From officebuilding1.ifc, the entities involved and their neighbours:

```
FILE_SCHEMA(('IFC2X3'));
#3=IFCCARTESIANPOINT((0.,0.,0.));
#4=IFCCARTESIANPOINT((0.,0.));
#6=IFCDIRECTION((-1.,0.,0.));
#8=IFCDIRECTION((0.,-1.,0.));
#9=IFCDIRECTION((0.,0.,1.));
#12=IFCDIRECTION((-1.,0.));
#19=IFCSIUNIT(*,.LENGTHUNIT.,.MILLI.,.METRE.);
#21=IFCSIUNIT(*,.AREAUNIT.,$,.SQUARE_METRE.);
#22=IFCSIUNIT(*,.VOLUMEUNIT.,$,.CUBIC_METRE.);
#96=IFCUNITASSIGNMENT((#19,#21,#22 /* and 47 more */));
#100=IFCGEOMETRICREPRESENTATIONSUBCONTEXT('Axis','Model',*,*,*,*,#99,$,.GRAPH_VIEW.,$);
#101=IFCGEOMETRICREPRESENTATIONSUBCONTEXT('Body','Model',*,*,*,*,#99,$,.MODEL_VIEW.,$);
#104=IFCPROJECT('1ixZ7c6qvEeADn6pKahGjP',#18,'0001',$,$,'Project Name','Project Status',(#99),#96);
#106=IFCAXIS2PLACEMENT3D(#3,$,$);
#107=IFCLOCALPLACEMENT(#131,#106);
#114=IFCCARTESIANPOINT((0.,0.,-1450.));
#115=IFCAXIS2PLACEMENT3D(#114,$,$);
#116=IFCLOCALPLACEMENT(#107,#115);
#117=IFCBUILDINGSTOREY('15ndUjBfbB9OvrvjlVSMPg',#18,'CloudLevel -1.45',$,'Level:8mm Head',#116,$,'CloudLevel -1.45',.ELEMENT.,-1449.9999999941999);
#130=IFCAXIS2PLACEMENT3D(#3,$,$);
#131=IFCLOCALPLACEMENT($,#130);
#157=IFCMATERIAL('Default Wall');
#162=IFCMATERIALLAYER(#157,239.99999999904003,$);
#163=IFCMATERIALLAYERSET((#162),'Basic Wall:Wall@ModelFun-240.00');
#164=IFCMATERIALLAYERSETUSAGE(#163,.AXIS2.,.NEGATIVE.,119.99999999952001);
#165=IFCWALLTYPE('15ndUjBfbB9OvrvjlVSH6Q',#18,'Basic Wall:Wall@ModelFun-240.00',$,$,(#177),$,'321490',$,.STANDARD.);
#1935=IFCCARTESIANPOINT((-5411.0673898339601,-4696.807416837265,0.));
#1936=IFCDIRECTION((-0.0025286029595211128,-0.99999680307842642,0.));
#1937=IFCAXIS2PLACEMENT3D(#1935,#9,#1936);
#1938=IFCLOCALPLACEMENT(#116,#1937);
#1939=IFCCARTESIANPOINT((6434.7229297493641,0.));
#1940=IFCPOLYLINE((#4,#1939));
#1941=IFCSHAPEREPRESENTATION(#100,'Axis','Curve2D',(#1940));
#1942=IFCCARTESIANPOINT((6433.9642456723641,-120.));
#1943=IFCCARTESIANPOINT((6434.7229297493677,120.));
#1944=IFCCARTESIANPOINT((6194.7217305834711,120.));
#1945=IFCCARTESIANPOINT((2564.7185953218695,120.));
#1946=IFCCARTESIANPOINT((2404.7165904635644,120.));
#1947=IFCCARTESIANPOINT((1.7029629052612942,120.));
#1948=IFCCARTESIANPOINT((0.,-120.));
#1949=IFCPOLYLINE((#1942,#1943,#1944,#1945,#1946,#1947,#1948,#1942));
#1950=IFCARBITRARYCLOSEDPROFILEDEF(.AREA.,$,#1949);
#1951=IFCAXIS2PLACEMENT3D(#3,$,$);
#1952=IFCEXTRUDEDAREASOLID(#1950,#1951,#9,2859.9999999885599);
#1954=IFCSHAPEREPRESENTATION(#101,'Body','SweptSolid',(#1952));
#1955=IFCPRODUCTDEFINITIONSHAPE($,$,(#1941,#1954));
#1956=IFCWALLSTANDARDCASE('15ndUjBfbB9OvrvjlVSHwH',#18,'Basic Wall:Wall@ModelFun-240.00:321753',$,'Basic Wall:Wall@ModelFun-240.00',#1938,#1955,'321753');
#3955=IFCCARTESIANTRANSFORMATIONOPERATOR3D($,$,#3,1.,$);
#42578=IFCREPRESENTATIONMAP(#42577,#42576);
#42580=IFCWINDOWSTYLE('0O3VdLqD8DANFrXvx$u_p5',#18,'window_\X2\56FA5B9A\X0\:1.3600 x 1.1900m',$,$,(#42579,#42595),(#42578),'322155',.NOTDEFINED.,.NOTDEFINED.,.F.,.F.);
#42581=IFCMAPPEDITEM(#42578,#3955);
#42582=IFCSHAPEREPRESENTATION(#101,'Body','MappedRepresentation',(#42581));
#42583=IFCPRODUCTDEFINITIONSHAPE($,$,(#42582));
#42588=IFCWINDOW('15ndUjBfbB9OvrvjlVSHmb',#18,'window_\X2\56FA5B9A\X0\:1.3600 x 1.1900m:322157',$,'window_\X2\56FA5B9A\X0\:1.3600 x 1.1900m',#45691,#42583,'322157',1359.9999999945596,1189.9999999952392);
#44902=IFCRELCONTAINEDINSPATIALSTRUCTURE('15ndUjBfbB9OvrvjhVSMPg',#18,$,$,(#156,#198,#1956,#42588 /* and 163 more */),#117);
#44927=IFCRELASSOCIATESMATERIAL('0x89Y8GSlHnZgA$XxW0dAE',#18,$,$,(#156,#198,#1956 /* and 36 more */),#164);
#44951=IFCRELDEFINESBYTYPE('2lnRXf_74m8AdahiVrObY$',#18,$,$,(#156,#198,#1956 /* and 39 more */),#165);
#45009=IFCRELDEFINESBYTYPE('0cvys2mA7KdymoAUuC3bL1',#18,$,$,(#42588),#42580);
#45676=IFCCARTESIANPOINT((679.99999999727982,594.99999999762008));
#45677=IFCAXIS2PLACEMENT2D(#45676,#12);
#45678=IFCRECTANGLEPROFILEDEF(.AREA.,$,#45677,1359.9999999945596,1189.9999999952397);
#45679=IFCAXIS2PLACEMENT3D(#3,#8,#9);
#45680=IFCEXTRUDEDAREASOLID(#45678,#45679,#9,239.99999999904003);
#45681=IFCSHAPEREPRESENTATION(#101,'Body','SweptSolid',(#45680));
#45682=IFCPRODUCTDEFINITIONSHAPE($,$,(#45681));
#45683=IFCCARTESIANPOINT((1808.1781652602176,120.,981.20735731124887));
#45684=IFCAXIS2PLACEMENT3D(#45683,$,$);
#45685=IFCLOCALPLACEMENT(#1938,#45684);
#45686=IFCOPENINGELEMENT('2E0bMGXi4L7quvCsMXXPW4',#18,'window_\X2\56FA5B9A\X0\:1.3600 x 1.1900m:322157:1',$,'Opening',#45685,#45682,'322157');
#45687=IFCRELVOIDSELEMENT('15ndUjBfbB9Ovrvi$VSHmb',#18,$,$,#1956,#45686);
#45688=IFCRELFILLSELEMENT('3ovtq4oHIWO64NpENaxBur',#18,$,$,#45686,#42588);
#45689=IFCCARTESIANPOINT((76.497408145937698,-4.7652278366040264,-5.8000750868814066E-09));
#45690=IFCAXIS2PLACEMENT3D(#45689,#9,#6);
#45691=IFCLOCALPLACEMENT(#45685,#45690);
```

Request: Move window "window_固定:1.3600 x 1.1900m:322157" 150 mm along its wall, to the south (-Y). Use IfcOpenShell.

```python
import ifcopenshell
import ifcopenshell.api.geometry
import ifcopenshell.util.placement

model = ifcopenshell.open("officebuilding1.ifc")

window = model.by_guid("15ndUjBfbB9OvrvjlVSHmb")
opening = window.FillsVoids[0].RelatingOpeningElement
wall = opening.VoidsElements[0].RelatingBuildingElement

wall_matrix = ifcopenshell.util.placement.get_local_placement(wall.ObjectPlacement)
shift = wall_matrix[:3, 0] * 150.0
before = ifcopenshell.util.placement.get_local_placement(window.ObjectPlacement)[:3, 3].copy()

# The window is placed relative to its opening, so it follows when the opening moves.
matrix = ifcopenshell.util.placement.get_local_placement(opening.ObjectPlacement)
matrix[:3, 3] += shift
ifcopenshell.api.geometry.edit_object_placement(
    model, product=opening, matrix=matrix, is_si=False, should_transform_children=True
)

after = ifcopenshell.util.placement.get_local_placement(window.ObjectPlacement)[:3, 3]
print("window moved by", (after - before).round(3) + 0.0)

model.write("officebuilding1_updated.ifc")
```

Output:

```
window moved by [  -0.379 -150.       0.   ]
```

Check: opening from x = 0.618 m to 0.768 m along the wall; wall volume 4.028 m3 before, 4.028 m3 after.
